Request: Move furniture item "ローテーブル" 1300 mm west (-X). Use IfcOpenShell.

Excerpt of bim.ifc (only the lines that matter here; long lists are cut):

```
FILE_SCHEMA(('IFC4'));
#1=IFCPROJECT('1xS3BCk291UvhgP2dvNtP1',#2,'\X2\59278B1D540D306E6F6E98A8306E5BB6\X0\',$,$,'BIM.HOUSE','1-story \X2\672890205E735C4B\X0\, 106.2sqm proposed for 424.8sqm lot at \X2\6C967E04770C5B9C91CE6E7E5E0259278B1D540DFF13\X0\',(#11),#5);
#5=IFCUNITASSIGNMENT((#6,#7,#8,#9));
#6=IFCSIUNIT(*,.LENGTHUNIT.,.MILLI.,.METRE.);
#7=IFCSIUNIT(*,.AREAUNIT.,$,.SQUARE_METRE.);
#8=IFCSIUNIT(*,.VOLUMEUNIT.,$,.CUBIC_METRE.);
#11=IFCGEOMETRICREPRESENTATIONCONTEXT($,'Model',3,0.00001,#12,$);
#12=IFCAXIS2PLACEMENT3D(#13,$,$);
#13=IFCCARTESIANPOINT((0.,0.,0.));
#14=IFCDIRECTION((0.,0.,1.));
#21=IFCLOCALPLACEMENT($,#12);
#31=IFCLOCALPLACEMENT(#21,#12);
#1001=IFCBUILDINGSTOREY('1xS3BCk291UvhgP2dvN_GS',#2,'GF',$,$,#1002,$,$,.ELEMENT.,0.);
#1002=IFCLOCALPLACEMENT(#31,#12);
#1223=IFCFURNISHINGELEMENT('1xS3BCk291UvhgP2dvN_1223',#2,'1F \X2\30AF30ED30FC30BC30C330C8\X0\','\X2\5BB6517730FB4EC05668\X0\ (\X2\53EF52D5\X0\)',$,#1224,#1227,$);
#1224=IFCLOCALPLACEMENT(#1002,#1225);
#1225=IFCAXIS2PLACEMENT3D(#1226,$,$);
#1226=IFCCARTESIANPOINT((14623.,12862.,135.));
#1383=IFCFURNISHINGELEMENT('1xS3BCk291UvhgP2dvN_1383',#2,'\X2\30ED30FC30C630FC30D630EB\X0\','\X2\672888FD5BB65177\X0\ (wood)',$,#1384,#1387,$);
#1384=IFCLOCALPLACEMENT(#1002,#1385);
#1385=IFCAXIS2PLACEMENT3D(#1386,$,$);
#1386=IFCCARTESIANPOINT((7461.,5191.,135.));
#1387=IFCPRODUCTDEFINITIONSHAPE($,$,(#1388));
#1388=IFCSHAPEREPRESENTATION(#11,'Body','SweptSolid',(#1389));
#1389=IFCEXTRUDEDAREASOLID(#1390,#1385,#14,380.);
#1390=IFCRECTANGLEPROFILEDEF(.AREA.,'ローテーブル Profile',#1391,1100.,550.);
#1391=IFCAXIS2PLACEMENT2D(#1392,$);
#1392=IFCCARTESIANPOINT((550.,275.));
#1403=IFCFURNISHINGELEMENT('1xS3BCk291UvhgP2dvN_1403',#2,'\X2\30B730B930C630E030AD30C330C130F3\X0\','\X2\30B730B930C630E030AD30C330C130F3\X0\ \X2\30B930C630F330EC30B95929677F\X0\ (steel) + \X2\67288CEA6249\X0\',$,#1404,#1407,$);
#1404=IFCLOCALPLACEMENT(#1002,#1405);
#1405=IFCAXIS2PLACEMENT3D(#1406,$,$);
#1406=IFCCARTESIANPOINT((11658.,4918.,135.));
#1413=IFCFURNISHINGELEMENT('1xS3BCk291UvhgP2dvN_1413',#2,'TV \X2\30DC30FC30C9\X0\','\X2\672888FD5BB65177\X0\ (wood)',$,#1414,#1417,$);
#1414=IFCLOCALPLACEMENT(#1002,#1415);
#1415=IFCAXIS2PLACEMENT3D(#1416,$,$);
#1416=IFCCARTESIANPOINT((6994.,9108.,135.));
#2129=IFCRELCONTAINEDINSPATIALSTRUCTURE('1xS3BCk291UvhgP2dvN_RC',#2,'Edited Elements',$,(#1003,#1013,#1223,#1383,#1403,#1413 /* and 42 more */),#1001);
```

```python
import ifcopenshell
import ifcopenshell.api.geometry
import ifcopenshell.util.placement

model = ifcopenshell.open("bim.ifc")

item = model.by_guid("1xS3BCk291UvhgP2dvN_1383")
matrix = ifcopenshell.util.placement.get_local_placement(item.ObjectPlacement)
matrix[0, 3] -= 1300.0
ifcopenshell.api.geometry.edit_object_placement(model, product=item, matrix=matrix, is_si=False)

print(ifcopenshell.util.placement.get_local_placement(item.ObjectPlacement).round(3) + 0.0)

model.write("bim-out.ifc")
```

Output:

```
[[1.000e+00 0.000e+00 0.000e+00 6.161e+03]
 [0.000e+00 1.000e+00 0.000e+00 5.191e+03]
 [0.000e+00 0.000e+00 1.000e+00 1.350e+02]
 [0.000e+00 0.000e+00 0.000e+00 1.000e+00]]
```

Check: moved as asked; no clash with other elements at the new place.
